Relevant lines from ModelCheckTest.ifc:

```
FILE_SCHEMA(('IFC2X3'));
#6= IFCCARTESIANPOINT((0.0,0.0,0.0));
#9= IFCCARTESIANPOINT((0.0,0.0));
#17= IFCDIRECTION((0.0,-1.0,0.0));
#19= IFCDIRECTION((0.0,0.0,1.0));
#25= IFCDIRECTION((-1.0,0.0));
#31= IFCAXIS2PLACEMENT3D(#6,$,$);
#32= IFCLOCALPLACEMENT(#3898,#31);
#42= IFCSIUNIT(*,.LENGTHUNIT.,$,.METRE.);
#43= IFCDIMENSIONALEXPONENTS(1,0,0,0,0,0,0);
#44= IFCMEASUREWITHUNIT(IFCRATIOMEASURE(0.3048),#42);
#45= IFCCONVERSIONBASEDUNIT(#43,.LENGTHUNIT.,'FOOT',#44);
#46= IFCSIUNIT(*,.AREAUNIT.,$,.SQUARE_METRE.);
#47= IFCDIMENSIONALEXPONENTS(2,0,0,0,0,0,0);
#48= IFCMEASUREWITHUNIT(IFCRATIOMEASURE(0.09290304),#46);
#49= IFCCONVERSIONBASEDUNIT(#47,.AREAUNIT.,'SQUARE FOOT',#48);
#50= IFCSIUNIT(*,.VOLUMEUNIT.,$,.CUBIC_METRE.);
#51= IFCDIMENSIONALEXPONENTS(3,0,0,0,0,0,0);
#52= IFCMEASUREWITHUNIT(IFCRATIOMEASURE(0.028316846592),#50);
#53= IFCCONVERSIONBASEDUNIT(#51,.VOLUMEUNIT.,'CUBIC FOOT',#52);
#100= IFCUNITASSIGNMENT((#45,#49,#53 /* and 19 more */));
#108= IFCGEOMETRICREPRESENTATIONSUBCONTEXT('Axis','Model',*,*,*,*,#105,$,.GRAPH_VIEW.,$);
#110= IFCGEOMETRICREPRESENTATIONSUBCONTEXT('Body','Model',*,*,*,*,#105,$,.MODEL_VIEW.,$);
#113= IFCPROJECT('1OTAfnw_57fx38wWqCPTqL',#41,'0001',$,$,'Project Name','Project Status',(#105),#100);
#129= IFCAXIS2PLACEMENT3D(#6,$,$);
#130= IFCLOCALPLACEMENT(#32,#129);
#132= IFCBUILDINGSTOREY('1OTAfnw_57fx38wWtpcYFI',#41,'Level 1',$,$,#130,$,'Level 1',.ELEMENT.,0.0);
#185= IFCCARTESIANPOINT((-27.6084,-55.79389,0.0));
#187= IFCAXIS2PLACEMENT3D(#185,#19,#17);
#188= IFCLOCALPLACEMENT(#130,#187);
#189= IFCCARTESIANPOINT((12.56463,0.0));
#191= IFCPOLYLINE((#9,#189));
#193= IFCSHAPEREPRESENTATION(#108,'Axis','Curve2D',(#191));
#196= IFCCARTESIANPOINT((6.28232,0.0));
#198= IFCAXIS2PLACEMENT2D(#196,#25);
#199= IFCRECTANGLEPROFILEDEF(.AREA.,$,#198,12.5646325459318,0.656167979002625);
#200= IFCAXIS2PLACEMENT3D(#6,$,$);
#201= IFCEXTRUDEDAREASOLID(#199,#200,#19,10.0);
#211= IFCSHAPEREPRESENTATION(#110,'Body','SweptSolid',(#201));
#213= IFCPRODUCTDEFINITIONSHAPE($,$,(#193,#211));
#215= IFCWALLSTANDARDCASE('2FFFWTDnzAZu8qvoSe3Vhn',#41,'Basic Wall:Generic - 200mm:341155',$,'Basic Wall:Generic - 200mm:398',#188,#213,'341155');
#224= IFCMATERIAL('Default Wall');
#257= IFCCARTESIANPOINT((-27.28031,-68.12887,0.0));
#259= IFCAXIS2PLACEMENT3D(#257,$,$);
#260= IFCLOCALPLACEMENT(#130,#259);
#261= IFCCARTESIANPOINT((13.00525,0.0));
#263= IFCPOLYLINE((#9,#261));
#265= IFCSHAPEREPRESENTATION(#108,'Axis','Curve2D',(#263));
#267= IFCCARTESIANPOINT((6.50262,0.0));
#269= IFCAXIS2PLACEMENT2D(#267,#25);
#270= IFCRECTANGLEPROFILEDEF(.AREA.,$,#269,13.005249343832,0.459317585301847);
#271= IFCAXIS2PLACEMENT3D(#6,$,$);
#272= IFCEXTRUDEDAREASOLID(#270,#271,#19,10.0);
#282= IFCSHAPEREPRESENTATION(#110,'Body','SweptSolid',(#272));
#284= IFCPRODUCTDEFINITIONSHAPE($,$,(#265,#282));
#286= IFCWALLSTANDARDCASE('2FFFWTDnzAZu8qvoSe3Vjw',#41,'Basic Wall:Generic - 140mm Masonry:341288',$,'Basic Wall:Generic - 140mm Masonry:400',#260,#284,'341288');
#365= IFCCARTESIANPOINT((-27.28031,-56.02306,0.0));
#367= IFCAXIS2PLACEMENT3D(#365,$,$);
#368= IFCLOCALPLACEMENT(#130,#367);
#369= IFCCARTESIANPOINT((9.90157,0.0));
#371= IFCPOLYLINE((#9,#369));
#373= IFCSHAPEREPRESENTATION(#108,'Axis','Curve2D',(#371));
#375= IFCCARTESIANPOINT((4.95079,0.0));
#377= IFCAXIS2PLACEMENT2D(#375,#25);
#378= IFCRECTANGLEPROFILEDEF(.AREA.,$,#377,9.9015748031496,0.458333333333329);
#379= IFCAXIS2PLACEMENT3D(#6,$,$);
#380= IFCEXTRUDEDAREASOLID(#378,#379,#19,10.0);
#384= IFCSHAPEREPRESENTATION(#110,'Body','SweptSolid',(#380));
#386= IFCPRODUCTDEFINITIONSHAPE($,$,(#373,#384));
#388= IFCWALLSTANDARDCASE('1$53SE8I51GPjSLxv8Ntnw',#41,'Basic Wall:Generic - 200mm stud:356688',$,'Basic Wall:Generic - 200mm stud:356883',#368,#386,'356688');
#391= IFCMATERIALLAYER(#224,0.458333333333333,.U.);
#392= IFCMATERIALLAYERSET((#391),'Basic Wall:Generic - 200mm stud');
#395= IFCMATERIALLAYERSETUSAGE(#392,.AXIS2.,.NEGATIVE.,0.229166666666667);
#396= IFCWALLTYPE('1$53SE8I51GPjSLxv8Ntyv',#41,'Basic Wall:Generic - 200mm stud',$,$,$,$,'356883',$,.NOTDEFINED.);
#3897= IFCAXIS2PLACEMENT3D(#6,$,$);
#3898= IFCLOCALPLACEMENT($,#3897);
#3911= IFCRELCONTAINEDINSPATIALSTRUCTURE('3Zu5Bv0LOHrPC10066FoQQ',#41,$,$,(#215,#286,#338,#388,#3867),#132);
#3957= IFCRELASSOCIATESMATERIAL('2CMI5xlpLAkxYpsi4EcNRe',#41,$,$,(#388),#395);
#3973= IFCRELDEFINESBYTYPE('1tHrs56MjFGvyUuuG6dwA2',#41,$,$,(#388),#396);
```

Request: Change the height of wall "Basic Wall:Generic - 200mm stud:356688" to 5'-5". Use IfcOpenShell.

```python
import ifcopenshell
import ifcopenshell.geom
import ifcopenshell.util.representation
import ifcopenshell.util.shape
import ifcopenshell.util.unit

model = ifcopenshell.open("ModelCheckTest.ifc")
unit_scale = ifcopenshell.util.unit.calculate_unit_scale(model)
settings = ifcopenshell.geom.settings()


def volume(element):
    """Net volume in cubic metres, openings subtracted."""
    shape = ifcopenshell.geom.create_shape(settings, element)
    return ifcopenshell.util.shape.get_volume(shape.geometry)


wall = model.by_guid("1$53SE8I51GPjSLxv8Ntnw")
before = volume(wall)

body = ifcopenshell.util.representation.get_representation(wall, "Model", "Body")
solid = body.Items[0]
old_height = solid.Depth
solid.Depth = 65 * 0.0254 / unit_scale
after = volume(wall)

print(f"height {old_height:g} -> {solid.Depth:g}, volume {before:.3f} -> {after:.3f} m3")

model.write("ModelCheckTest_updated.ifc")
```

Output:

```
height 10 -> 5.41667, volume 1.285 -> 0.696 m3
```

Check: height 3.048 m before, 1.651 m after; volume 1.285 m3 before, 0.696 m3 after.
